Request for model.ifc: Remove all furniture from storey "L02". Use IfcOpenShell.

First a look at what the model holds.

```python
import ifcopenshell
import ifcopenshell.util.element

model = ifcopenshell.open("model.ifc")
print(model.schema)
storey = next(s for s in model.by_type("IfcBuildingStorey") if s.Name == "L02")
furniture = [e for e in ifcopenshell.util.element.get_decomposition(storey) if e.is_a("IfcFurnishingElement")]
seen = {}
for e in furniture:
    element_type = ifcopenshell.util.element.get_type(e)
    name = element_type.Name if element_type not in (None, e) else None
    seen[name] = seen.get(name, 0) + 1
for name, count in sorted(seen.items(), key=str):
    print(count, "x", name)
```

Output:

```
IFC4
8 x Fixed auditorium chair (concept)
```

```python
import ifcopenshell
import ifcopenshell.api.root
import ifcopenshell.util.element

model = ifcopenshell.open("model.ifc")

storey = next(s for s in model.by_type("IfcBuildingStorey") if s.Name == "L02")
furniture = [e for e in ifcopenshell.util.element.get_decomposition(storey) if e.is_a("IfcFurnishingElement")]

for e in furniture:
    ifcopenshell.api.root.remove_product(model, product=e)
print(len(furniture), "removed")

model.write("model_rev.ifc")
```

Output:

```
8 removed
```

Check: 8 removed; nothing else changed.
